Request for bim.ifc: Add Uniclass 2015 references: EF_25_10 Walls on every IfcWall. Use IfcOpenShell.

First a look at what the model holds.

```python
import ifcopenshell

model = ifcopenshell.open("bim.ifc")
print(model.schema)
print("classifications:", [c.Name for c in model.by_type("IfcClassification")])
for ifc_class in ("IfcDoor", "IfcRoof", "IfcStair", "IfcWall", "IfcWindow"):
    print(ifc_class, len(model.by_type(ifc_class)))
```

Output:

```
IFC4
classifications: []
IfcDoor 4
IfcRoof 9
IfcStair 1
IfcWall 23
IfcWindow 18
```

```python
import ifcopenshell
import ifcopenshell.api.classification

model = ifcopenshell.open("bim.ifc")

system = ifcopenshell.api.classification.add_classification(model, classification="Uniclass 2015")

codes = {
    "IfcWall": ("EF_25_10", "Walls"),
}
for ifc_class, (code, name) in codes.items():
    products = model.by_type(ifc_class)
    ifcopenshell.api.classification.add_reference(
        model, products=products, classification=system, identification=code, name=name
    )
    print(code, len(products))

model.write("bim_edited.ifc")
```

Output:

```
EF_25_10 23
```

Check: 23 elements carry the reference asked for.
